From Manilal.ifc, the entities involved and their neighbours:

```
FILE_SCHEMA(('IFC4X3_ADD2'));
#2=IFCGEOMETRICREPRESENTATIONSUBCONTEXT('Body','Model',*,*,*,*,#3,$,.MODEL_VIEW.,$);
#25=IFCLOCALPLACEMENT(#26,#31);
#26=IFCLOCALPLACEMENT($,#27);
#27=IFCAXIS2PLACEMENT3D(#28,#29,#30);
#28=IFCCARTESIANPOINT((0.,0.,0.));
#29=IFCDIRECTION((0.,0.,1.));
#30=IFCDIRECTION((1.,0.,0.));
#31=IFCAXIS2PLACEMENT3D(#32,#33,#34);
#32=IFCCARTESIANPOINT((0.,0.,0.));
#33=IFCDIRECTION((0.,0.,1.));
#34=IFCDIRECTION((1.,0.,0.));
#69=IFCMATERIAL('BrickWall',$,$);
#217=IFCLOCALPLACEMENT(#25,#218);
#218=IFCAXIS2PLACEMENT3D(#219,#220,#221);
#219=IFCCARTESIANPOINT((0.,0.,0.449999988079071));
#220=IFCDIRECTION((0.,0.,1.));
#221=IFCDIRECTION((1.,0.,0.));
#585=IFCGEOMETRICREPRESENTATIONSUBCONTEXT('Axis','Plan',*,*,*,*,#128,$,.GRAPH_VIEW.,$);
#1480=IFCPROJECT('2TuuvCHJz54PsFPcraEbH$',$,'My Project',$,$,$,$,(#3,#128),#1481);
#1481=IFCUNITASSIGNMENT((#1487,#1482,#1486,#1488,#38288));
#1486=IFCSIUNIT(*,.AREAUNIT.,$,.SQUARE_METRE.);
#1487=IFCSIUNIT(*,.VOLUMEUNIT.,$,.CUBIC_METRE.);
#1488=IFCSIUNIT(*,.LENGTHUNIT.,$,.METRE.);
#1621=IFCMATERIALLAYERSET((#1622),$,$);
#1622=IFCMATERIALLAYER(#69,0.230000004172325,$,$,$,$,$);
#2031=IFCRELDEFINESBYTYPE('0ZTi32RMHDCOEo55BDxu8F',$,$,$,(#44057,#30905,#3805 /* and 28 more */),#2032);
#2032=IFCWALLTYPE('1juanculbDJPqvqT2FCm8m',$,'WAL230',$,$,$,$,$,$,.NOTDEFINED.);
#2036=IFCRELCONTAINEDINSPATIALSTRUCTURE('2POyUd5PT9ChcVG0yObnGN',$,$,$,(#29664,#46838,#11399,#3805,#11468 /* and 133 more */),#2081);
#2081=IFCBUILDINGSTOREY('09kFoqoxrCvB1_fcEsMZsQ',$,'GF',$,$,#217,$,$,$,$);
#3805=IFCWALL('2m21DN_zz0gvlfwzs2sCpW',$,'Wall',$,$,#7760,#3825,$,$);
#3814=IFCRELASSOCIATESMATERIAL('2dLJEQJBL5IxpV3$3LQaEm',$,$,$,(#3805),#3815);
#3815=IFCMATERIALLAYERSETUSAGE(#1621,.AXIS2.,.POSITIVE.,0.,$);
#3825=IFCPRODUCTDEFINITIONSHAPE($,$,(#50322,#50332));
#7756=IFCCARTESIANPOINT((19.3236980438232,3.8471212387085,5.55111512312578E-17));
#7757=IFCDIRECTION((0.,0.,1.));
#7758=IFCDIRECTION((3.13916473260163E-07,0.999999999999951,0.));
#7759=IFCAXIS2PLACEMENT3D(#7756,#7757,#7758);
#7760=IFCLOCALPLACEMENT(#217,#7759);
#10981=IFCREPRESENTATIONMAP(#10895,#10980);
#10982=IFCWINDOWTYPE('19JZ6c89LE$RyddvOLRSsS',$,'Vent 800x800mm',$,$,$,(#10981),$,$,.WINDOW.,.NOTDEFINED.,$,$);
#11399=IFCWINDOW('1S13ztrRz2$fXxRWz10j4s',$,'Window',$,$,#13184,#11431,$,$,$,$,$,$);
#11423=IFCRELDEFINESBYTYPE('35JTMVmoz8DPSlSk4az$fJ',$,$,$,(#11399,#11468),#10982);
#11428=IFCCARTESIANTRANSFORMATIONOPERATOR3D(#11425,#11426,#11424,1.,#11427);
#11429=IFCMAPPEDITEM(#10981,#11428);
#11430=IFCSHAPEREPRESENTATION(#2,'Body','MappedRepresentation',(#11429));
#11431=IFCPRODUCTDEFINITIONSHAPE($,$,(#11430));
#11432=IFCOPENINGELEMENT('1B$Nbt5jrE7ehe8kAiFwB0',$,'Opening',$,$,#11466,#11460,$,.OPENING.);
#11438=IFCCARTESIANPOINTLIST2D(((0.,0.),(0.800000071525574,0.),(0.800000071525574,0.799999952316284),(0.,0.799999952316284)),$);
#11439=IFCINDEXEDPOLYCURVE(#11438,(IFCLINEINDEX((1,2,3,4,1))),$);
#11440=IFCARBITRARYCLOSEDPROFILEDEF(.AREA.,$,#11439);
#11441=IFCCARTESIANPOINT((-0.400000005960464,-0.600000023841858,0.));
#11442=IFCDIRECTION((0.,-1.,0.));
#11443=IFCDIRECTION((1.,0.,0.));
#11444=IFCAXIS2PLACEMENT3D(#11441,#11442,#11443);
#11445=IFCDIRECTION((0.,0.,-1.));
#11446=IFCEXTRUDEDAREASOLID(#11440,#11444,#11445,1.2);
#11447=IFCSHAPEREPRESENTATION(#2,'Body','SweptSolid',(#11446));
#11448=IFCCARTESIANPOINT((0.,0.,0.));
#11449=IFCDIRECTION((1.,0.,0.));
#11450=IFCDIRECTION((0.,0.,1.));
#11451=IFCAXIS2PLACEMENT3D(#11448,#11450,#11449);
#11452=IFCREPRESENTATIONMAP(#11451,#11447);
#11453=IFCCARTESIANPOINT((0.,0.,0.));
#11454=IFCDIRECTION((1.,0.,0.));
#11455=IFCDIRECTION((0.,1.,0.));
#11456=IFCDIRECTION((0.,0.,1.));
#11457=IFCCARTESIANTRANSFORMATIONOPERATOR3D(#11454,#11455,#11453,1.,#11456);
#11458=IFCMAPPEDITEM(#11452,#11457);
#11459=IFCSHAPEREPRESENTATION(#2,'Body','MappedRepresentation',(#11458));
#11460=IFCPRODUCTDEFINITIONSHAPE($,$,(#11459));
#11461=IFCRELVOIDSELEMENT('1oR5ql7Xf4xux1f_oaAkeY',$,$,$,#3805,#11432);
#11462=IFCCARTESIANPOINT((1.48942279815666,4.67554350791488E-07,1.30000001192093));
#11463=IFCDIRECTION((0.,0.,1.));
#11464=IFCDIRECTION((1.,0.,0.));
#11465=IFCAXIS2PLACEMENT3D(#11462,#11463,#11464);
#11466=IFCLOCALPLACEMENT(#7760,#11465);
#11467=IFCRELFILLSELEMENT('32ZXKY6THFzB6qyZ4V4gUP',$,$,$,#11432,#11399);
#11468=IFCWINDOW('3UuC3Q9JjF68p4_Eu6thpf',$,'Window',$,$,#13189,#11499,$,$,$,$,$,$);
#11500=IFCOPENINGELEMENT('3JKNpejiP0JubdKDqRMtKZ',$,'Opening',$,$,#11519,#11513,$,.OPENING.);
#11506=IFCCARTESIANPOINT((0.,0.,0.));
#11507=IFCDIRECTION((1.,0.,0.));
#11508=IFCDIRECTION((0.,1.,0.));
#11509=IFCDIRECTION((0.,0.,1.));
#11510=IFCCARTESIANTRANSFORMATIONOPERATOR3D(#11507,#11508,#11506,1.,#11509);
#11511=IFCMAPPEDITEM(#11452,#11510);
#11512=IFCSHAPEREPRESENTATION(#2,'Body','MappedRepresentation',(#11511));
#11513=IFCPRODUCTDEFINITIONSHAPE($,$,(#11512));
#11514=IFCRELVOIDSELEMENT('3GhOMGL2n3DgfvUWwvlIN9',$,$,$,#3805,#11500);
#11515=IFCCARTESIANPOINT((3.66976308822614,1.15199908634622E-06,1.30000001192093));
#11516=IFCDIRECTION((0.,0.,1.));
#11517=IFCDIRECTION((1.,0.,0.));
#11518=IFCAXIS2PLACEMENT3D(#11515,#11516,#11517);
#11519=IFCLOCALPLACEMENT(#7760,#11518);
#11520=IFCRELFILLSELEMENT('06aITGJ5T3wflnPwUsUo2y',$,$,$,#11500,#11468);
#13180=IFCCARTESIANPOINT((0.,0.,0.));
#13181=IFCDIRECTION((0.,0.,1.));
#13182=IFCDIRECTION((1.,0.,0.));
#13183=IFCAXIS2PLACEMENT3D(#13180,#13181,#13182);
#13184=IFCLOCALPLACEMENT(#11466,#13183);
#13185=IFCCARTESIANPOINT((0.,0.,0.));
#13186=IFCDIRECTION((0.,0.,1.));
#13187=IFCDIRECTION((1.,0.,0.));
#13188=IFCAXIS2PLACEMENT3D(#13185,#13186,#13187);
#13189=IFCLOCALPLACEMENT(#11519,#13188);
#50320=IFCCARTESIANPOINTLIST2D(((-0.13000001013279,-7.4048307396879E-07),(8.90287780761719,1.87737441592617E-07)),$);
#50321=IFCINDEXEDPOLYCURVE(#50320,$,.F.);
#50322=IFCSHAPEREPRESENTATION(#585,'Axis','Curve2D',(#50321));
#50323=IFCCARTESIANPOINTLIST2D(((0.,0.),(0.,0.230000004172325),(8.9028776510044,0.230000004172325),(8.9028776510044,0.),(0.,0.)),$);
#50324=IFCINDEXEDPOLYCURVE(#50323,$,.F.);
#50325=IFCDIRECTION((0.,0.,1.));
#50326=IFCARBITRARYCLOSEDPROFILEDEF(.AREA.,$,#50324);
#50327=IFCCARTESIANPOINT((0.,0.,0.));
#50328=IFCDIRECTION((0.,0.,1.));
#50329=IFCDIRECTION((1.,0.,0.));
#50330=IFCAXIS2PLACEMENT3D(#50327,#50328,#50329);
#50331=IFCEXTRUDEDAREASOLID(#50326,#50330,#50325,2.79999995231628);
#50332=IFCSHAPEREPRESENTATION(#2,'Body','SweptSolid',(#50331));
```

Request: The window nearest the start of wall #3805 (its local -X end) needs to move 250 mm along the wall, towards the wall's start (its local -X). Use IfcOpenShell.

```python
import ifcopenshell
import ifcopenshell.api.geometry
import ifcopenshell.util.placement

model = ifcopenshell.open("Manilal.ifc")

window = model.by_guid("1S13ztrRz2$fXxRWz10j4s")
opening = window.FillsVoids[0].RelatingOpeningElement
wall = opening.VoidsElements[0].RelatingBuildingElement

wall_matrix = ifcopenshell.util.placement.get_local_placement(wall.ObjectPlacement)
shift = wall_matrix[:3, 0] * -0.25
before = ifcopenshell.util.placement.get_local_placement(window.ObjectPlacement)[:3, 3].copy()

# The window is placed relative to its opening, so it follows when the opening moves.
matrix = ifcopenshell.util.placement.get_local_placement(opening.ObjectPlacement)
matrix[:3, 3] += shift
ifcopenshell.api.geometry.edit_object_placement(
    model, product=opening, matrix=matrix, is_si=False, should_transform_children=True
)

after = ifcopenshell.util.placement.get_local_placement(window.ObjectPlacement)[:3, 3]
print("window moved by", (after - before).round(3) + 0.0)

model.write("Manilal_updated.ifc")
```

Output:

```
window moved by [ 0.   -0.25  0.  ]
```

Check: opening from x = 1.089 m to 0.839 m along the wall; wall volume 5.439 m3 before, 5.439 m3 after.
